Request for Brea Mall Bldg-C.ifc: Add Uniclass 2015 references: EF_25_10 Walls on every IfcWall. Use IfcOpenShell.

First a look at what the model holds.

```python
import ifcopenshell

model = ifcopenshell.open("Brea Mall Bldg-C.ifc")
print(model.schema)
print("classifications:", [c.Name for c in model.by_type("IfcClassification")])
for ifc_class in ("IfcDoor", "IfcRoof", "IfcStair", "IfcWall", "IfcWindow"):
    print(ifc_class, len(model.by_type(ifc_class)))
```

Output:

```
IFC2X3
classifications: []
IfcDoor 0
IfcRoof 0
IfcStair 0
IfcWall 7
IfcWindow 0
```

```python
import ifcopenshell
import ifcopenshell.api.classification

model = ifcopenshell.open("Brea Mall Bldg-C.ifc")

# IFC2X3 requires Source and Edition and has no link from the project to the system.
system = model.create_entity("IfcClassification", Source="NBS", Edition="2015", Name="Uniclass 2015")

codes = {
    "IfcWall": ("EF_25_10", "Walls"),
}
for ifc_class, (code, name) in codes.items():
    products = model.by_type(ifc_class)
    ifcopenshell.api.classification.add_reference(
        model, products=products, classification=system, identification=code, name=name
    )
    print(code, len(products))

model.write("Brea Mall Bldg-C_v2.ifc")
```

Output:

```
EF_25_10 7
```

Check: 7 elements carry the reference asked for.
